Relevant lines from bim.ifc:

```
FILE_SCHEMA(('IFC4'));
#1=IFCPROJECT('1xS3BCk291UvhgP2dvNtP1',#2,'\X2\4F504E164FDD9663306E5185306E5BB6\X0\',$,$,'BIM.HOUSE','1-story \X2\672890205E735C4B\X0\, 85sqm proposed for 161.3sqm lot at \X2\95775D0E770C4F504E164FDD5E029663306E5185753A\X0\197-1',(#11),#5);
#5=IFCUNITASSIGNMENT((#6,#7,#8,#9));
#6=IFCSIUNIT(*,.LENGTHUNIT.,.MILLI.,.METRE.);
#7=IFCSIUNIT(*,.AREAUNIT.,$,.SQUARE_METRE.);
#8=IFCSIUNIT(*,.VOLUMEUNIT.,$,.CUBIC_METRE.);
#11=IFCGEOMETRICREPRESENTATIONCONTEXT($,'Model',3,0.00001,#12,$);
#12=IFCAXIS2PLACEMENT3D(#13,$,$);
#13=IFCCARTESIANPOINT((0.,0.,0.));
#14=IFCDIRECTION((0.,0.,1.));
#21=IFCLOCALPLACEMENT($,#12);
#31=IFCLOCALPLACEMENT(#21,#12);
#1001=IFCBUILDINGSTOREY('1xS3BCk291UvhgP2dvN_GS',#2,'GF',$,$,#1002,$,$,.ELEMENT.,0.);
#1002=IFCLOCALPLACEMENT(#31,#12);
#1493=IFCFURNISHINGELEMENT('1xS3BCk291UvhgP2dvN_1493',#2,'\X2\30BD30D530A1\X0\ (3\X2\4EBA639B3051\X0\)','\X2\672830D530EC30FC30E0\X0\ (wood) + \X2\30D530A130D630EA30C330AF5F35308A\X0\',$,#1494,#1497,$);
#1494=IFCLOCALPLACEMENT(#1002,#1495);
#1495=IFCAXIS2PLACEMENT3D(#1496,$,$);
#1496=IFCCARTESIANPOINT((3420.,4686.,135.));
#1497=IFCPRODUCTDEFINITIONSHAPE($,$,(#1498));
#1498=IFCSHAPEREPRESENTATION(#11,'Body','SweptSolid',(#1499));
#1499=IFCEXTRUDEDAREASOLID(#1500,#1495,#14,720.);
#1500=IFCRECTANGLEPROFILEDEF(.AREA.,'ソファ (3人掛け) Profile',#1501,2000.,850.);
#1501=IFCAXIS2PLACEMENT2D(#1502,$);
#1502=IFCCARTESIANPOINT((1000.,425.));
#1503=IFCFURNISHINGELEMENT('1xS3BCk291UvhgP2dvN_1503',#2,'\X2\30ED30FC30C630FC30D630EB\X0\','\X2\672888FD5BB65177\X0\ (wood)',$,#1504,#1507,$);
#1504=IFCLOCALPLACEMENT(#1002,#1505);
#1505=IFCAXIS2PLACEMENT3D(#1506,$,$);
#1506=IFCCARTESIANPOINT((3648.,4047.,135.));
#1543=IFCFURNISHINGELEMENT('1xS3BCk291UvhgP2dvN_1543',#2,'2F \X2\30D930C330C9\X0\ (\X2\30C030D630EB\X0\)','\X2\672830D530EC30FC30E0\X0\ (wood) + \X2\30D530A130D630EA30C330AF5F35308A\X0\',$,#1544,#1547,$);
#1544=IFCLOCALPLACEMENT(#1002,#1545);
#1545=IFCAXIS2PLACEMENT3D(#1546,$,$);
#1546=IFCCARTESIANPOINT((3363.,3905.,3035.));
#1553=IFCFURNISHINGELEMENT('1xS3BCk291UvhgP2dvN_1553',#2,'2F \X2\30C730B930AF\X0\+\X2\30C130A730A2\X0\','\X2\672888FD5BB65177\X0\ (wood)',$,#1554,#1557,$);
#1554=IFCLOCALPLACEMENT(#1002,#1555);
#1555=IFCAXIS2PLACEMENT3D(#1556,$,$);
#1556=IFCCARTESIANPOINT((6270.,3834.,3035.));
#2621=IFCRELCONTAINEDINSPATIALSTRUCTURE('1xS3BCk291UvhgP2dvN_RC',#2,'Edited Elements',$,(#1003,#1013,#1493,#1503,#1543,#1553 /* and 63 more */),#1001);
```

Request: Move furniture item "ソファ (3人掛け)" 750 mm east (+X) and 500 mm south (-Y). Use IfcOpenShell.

```python
import ifcopenshell
import ifcopenshell.api.geometry
import ifcopenshell.util.placement

model = ifcopenshell.open("bim.ifc")

item = model.by_guid("1xS3BCk291UvhgP2dvN_1493")
matrix = ifcopenshell.util.placement.get_local_placement(item.ObjectPlacement)
matrix[0, 3] += 750.0
matrix[1, 3] -= 500.0
ifcopenshell.api.geometry.edit_object_placement(model, product=item, matrix=matrix, is_si=False)

print(ifcopenshell.util.placement.get_local_placement(item.ObjectPlacement).round(3) + 0.0)

model.write("bim_rev.ifc")
```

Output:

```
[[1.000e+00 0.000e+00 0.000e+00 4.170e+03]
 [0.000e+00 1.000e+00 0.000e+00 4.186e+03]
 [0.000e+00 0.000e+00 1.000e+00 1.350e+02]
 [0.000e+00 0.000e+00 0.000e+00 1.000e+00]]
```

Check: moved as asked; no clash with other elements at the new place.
